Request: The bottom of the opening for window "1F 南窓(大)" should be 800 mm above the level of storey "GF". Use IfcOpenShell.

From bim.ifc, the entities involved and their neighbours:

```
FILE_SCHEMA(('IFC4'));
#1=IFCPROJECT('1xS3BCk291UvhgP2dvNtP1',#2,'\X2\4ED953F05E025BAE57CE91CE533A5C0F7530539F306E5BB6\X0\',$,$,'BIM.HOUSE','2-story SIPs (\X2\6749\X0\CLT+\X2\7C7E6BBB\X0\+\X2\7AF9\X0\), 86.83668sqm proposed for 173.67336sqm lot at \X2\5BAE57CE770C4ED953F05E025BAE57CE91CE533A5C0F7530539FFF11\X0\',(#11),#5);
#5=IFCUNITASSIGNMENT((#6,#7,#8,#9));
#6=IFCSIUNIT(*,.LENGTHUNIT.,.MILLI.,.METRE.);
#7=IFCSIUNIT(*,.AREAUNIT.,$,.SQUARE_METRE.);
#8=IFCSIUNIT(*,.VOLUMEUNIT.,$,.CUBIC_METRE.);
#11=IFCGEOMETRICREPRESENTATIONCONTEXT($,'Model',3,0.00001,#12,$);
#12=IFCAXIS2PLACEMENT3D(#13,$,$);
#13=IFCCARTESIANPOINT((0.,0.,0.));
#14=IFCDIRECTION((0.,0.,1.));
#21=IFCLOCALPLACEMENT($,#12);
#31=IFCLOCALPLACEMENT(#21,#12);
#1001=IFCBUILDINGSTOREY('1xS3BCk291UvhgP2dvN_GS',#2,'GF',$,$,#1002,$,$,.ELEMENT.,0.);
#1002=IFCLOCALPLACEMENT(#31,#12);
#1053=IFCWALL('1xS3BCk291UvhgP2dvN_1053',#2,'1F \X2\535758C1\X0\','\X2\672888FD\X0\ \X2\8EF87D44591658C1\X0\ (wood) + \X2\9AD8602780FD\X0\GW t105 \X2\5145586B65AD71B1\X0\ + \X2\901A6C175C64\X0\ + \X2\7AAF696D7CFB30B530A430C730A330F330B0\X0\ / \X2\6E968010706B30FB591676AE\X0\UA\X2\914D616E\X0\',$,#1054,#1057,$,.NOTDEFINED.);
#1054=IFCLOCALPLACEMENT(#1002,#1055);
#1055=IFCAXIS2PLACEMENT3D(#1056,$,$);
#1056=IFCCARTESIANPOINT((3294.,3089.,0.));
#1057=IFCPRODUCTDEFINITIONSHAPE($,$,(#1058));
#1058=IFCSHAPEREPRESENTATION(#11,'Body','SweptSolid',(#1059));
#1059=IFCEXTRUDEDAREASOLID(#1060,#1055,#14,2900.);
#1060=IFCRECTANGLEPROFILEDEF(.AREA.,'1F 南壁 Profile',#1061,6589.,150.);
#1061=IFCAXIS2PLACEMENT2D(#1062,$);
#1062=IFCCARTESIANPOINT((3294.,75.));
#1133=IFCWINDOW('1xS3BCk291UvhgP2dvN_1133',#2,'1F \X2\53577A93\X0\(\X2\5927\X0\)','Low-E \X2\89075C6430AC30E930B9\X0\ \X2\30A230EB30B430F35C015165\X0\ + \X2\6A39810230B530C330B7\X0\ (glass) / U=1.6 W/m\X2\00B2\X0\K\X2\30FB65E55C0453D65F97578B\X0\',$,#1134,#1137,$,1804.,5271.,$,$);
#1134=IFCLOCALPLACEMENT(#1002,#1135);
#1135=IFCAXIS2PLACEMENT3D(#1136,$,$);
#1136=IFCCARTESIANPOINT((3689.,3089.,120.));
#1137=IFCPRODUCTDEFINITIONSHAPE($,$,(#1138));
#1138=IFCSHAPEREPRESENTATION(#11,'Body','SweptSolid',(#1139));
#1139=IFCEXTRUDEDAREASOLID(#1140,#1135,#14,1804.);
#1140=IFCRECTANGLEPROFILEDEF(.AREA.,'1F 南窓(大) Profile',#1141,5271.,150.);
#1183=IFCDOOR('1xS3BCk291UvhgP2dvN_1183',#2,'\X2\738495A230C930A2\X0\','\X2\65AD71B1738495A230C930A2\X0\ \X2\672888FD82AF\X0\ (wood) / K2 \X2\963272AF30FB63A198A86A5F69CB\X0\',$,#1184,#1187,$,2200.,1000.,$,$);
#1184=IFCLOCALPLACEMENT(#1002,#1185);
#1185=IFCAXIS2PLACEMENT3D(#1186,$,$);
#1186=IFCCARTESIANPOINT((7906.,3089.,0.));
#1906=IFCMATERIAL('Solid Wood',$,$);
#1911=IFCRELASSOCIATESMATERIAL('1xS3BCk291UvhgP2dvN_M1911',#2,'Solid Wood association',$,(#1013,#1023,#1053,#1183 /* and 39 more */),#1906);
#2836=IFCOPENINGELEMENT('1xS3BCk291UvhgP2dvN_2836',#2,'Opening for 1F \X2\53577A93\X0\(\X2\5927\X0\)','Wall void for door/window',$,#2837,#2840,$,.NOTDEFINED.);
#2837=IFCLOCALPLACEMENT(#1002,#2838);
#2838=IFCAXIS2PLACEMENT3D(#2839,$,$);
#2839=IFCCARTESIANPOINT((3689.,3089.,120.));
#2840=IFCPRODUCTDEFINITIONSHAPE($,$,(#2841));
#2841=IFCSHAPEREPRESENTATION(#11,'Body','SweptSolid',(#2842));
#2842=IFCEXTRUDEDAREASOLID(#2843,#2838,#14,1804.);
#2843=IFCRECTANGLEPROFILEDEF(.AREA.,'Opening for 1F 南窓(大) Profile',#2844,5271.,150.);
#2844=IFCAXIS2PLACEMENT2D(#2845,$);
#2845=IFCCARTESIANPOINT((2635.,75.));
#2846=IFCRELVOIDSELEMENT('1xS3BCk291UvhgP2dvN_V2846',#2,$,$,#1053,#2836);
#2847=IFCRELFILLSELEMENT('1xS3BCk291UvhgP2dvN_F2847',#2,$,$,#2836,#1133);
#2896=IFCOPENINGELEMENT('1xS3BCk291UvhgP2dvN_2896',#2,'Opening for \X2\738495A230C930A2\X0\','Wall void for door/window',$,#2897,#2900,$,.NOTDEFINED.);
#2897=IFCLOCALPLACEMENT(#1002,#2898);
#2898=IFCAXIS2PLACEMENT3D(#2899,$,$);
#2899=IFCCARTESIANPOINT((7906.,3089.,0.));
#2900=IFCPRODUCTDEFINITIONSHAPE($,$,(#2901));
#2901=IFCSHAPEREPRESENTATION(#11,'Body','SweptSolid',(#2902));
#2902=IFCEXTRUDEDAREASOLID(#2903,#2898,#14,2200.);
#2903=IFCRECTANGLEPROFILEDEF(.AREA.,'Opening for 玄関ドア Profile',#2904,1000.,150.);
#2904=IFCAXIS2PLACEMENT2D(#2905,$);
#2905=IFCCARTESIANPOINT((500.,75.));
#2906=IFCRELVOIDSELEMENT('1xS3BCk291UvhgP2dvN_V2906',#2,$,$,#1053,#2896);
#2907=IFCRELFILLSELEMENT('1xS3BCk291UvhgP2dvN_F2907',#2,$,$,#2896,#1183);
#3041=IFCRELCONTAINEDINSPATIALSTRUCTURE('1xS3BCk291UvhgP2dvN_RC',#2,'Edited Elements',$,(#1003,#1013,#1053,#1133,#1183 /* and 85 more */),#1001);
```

```python
import numpy as np
import ifcopenshell
import ifcopenshell.api.geometry
import ifcopenshell.geom
import ifcopenshell.util.element
import ifcopenshell.util.placement
import ifcopenshell.util.shape
import ifcopenshell.util.unit

model = ifcopenshell.open("bim.ifc")
unit_scale = ifcopenshell.util.unit.calculate_unit_scale(model)

window = model.by_guid("1xS3BCk291UvhgP2dvN_1133")
opening = window.FillsVoids[0].RelatingOpeningElement
storey = ifcopenshell.util.element.get_container(window, ifc_class="IfcBuildingStorey")
level = ifcopenshell.util.placement.get_local_placement(storey.ObjectPlacement)[2, 3]

# The opening's origin need not be at the sill, so measure its lowest point.
shape = ifcopenshell.geom.create_shape(ifcopenshell.geom.settings(), opening)
bottom = ifcopenshell.util.shape.get_shape_bottom_elevation(shape, shape.geometry) / unit_scale
dz = level + 0.8 / unit_scale - bottom

shift = np.array([0.0, 0.0, dz])
# The window is not placed relative to its opening, so move both.
for product in (opening, window):
    matrix = ifcopenshell.util.placement.get_local_placement(product.ObjectPlacement)
    matrix[:3, 3] += shift
    ifcopenshell.api.geometry.edit_object_placement(model, product=product, matrix=matrix, is_si=False)

print(f"moved by {dz * unit_scale:+.3f} m")

model.write("bim_updated.ifc")
```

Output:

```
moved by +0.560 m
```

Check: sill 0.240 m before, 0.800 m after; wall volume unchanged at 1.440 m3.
